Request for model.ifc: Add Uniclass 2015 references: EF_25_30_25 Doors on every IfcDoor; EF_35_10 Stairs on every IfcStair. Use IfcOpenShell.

First a look at what the model holds.

```python
import ifcopenshell

model = ifcopenshell.open("model.ifc")
print(model.schema)
print("classifications:", [c.Name for c in model.by_type("IfcClassification")])
for ifc_class in ("IfcDoor", "IfcRoof", "IfcStair", "IfcWall", "IfcWindow"):
    print(ifc_class, len(model.by_type(ifc_class)))
```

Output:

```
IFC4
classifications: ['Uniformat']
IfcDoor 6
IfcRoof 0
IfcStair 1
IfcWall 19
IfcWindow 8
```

```python
import ifcopenshell
import ifcopenshell.api.classification

model = ifcopenshell.open("model.ifc")

system = ifcopenshell.api.classification.add_classification(model, classification="Uniclass 2015")

codes = {
    "IfcDoor": ("EF_25_30_25", "Doors"),
    "IfcStair": ("EF_35_10", "Stairs"),
}
for ifc_class, (code, name) in codes.items():
    products = model.by_type(ifc_class)
    ifcopenshell.api.classification.add_reference(
        model, products=products, classification=system, identification=code, name=name
    )
    print(code, len(products))

model.write("model_rev.ifc")
```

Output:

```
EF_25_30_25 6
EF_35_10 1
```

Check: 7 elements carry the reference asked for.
